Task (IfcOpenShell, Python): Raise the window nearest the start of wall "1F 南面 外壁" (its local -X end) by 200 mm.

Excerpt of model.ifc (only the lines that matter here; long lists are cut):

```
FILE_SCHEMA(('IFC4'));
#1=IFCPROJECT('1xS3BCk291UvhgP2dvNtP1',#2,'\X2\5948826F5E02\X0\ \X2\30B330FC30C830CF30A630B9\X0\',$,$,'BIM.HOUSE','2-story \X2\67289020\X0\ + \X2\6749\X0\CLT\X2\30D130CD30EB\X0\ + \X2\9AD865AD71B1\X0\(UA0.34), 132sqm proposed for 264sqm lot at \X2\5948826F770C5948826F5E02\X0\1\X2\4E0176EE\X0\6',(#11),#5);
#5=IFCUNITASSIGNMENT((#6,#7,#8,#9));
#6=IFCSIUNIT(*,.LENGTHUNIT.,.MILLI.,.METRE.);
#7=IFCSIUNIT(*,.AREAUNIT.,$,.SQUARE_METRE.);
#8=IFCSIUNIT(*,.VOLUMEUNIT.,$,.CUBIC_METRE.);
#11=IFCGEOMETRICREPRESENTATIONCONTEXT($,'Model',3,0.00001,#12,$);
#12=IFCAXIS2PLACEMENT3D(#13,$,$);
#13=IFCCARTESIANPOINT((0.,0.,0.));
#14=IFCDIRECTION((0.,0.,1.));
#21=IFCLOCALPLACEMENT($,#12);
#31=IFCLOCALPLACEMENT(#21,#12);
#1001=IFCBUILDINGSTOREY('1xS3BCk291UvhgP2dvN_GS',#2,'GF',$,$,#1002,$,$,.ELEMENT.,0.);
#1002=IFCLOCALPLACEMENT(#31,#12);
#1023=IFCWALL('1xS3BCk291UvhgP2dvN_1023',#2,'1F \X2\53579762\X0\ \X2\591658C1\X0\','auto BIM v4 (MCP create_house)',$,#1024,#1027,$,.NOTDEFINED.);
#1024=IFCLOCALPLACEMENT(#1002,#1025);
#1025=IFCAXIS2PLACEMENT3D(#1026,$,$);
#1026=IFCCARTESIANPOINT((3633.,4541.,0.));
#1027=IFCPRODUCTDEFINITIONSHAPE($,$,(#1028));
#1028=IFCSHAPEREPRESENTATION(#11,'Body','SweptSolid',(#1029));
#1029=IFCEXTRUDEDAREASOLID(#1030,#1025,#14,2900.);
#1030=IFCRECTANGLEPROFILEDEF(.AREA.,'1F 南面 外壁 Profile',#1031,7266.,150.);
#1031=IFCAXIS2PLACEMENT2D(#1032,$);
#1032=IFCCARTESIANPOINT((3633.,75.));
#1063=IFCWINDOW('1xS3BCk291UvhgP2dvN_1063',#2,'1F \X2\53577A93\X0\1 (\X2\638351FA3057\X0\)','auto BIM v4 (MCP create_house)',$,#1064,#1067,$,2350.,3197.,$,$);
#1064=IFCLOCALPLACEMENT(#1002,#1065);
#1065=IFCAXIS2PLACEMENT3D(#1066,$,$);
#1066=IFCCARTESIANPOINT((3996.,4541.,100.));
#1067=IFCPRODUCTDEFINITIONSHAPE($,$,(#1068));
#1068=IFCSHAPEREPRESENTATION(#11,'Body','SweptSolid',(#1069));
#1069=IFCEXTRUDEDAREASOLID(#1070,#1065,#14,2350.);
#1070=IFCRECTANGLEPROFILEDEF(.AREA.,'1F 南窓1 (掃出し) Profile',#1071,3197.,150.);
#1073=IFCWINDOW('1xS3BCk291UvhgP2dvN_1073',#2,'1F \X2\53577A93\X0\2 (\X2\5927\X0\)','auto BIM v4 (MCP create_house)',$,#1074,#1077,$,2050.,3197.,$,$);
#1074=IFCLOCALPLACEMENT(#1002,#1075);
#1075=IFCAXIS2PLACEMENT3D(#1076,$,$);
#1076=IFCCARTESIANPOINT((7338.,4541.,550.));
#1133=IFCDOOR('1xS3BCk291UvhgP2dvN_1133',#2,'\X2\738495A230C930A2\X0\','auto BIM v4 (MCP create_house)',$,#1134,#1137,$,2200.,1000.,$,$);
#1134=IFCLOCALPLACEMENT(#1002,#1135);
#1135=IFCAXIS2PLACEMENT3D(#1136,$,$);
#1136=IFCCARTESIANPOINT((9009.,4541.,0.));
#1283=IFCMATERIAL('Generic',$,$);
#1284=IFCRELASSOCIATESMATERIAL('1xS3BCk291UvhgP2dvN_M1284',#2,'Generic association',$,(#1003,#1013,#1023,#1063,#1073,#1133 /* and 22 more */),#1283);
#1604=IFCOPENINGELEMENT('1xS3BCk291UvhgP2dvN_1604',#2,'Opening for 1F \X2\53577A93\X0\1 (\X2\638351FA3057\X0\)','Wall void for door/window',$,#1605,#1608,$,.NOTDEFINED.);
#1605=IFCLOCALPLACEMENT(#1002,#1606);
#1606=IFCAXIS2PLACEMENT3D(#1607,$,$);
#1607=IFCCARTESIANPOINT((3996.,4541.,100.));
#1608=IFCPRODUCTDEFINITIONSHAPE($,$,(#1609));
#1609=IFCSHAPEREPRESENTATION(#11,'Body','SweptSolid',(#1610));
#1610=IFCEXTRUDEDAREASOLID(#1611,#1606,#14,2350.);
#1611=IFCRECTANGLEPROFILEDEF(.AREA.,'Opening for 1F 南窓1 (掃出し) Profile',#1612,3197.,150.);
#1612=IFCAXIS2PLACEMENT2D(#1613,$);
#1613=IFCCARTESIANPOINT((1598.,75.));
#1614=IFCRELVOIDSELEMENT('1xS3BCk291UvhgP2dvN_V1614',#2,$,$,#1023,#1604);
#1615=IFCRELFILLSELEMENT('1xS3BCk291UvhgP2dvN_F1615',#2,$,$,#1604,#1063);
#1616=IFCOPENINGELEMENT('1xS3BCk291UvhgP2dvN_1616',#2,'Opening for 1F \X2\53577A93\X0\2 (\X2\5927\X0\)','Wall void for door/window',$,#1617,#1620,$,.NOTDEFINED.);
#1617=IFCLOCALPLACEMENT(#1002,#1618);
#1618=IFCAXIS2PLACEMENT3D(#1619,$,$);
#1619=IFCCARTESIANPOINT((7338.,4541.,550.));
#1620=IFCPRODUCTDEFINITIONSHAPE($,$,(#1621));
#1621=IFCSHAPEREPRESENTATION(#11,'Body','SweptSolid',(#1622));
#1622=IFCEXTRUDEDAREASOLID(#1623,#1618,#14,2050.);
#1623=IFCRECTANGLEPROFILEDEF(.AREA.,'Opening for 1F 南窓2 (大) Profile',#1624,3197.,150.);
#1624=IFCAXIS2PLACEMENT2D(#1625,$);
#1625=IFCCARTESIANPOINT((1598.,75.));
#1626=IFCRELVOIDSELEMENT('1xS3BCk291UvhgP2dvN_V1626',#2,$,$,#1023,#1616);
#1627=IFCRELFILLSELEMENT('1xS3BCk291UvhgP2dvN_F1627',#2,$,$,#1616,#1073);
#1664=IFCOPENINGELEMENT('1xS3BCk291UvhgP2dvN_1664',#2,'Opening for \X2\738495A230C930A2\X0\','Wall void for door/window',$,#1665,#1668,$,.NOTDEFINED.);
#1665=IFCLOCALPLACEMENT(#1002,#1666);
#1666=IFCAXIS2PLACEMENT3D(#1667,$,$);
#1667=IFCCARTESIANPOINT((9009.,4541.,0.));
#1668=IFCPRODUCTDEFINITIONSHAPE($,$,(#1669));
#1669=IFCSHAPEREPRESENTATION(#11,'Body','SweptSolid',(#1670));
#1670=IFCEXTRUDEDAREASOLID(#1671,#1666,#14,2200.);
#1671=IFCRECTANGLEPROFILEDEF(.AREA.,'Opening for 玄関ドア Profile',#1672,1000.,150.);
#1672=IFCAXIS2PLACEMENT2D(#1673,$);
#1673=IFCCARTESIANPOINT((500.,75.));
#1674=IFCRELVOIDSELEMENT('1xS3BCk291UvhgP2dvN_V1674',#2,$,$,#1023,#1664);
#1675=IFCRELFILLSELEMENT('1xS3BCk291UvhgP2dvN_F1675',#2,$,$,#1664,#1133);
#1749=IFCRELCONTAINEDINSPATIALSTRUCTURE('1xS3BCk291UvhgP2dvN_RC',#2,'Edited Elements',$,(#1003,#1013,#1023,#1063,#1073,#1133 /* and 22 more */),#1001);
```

```python
import numpy as np
import ifcopenshell
import ifcopenshell.api.geometry
import ifcopenshell.util.placement
import ifcopenshell.util.unit

model = ifcopenshell.open("model.ifc")
unit_scale = ifcopenshell.util.unit.calculate_unit_scale(model)

window = model.by_guid("1xS3BCk291UvhgP2dvN_1063")
opening = window.FillsVoids[0].RelatingOpeningElement
dz = 0.2 / unit_scale

shift = np.array([0.0, 0.0, dz])
# The window is not placed relative to its opening, so move both.
for product in (opening, window):
    matrix = ifcopenshell.util.placement.get_local_placement(product.ObjectPlacement)
    matrix[:3, 3] += shift
    ifcopenshell.api.geometry.edit_object_placement(model, product=product, matrix=matrix, is_si=False)

print(f"moved by {dz * unit_scale:+.3f} m")

model.write("model_edited.ifc")
```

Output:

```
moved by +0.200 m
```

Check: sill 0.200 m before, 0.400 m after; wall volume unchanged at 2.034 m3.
